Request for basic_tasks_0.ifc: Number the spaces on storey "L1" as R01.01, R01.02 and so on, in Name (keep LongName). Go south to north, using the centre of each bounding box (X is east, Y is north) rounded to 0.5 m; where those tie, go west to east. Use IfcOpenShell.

First a look at what the model holds.

```python
import ifcopenshell
import ifcopenshell.util.element
import ifcopenshell.util.placement

model = ifcopenshell.open("basic_tasks_0.ifc")
print(model.schema)
storey = next(s for s in model.by_type("IfcBuildingStorey") if s.Name == "L1")
spaces = [e for e in ifcopenshell.util.element.get_decomposition(storey) if e.is_a("IfcSpace")]
for e in sorted(spaces, key=lambda e: e.id()):
    origin = ifcopenshell.util.placement.get_local_placement(e.ObjectPlacement)[:3, 3]
    print(e.id(), e.Name, e.LongName, origin.round(2) + 0.0, sep=" | ")
```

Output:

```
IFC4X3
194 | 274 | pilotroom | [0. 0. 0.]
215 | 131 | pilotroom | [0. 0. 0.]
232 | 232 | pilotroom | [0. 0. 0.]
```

```python
import ifcopenshell
import ifcopenshell.geom
import ifcopenshell.util.element
import ifcopenshell.util.shape

model = ifcopenshell.open("basic_tasks_0.ifc")
settings = ifcopenshell.geom.settings()
settings.set("use-world-coords", True)


def centre(element):
    shape = ifcopenshell.geom.create_shape(settings, element)
    return ifcopenshell.util.shape.get_bbox_centroid(shape.geometry)


storey = next(s for s in model.by_type("IfcBuildingStorey") if s.Name == "L1")
spaces = [e for e in ifcopenshell.util.element.get_decomposition(storey) if e.is_a("IfcSpace")]

# Insertion points can sit at a corner or the storey origin, so sort by the geometry (in metres).
centres = {e: centre(e) for e in spaces}
spaces.sort(key=lambda e: (round(centres[e][1] / 0.5), centres[e][0]))

for i, e in enumerate(spaces, start=1):
    number = f"R01.{i:02d}"
    e.Name = number
    print(e.id(), number)

model.write("basic_tasks_0_v2.ifc")
```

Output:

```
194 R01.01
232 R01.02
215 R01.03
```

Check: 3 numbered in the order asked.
